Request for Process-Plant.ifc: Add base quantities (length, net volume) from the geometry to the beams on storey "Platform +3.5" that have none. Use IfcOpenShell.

First a look at what the model holds.

```python
import ifcopenshell
import ifcopenshell.util.element
import ifcopenshell.util.unit

model = ifcopenshell.open("Process-Plant.ifc")
print(model.schema)
for unit_type in ("LENGTHUNIT", "AREAUNIT", "VOLUMEUNIT"):
    print(unit_type, ifcopenshell.util.unit.calculate_unit_scale(model, unit_type))
storey = next(s for s in model.by_type("IfcBuildingStorey") if s.Name == "Platform +3.5")
beams = [e for e in ifcopenshell.util.element.get_decomposition(storey) if e.is_a("IfcBeam")]
for e in sorted(beams, key=lambda e: e.id()):
    print(e.id(), e.is_a(), e.Name, list(ifcopenshell.util.element.get_psets(e, qtos_only=True)), sep=" | ")
```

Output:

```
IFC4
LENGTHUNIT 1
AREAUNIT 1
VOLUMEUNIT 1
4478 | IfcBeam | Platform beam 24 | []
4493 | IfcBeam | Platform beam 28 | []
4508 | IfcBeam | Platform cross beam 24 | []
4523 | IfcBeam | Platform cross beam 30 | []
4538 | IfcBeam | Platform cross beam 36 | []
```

```python
import ifcopenshell
import ifcopenshell.api.pset
import ifcopenshell.geom
import ifcopenshell.util.element
import ifcopenshell.util.shape
import ifcopenshell.util.unit

model = ifcopenshell.open("Process-Plant.ifc")
unit_scale = ifcopenshell.util.unit.calculate_unit_scale(model)
volume_scale = ifcopenshell.util.unit.calculate_unit_scale(model, "VOLUMEUNIT")
settings = ifcopenshell.geom.settings()

storey = next(s for s in model.by_type("IfcBuildingStorey") if s.Name == "Platform +3.5")
beams = [e for e in ifcopenshell.util.element.get_decomposition(storey) if e.is_a("IfcBeam")]

for e in sorted(beams, key=lambda e: e.id()):
    if ifcopenshell.util.element.get_psets(e, qtos_only=True, should_inherit=False):
        continue
    # Geometry comes back in metres, in the element's own axes.
    shape = ifcopenshell.geom.create_shape(settings, e)
    values = {
        "Length": ifcopenshell.util.shape.get_max_xyz(shape.geometry) / unit_scale,
        "NetVolume": ifcopenshell.util.shape.get_volume(shape.geometry) / volume_scale,
    }
    qto = ifcopenshell.api.pset.add_qto(model, product=e, name="Qto_BeamBaseQuantities")
    ifcopenshell.api.pset.edit_qto(model, qto=qto, properties=values)
    print(e.id(), {k: round(v, 3) for k, v in values.items()})

model.write("Process-Plant-out.ifc")
```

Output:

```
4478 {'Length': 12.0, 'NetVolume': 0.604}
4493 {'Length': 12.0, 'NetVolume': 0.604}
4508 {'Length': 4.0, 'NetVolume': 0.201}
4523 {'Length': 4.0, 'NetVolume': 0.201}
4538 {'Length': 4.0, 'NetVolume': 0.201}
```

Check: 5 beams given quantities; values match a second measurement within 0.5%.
